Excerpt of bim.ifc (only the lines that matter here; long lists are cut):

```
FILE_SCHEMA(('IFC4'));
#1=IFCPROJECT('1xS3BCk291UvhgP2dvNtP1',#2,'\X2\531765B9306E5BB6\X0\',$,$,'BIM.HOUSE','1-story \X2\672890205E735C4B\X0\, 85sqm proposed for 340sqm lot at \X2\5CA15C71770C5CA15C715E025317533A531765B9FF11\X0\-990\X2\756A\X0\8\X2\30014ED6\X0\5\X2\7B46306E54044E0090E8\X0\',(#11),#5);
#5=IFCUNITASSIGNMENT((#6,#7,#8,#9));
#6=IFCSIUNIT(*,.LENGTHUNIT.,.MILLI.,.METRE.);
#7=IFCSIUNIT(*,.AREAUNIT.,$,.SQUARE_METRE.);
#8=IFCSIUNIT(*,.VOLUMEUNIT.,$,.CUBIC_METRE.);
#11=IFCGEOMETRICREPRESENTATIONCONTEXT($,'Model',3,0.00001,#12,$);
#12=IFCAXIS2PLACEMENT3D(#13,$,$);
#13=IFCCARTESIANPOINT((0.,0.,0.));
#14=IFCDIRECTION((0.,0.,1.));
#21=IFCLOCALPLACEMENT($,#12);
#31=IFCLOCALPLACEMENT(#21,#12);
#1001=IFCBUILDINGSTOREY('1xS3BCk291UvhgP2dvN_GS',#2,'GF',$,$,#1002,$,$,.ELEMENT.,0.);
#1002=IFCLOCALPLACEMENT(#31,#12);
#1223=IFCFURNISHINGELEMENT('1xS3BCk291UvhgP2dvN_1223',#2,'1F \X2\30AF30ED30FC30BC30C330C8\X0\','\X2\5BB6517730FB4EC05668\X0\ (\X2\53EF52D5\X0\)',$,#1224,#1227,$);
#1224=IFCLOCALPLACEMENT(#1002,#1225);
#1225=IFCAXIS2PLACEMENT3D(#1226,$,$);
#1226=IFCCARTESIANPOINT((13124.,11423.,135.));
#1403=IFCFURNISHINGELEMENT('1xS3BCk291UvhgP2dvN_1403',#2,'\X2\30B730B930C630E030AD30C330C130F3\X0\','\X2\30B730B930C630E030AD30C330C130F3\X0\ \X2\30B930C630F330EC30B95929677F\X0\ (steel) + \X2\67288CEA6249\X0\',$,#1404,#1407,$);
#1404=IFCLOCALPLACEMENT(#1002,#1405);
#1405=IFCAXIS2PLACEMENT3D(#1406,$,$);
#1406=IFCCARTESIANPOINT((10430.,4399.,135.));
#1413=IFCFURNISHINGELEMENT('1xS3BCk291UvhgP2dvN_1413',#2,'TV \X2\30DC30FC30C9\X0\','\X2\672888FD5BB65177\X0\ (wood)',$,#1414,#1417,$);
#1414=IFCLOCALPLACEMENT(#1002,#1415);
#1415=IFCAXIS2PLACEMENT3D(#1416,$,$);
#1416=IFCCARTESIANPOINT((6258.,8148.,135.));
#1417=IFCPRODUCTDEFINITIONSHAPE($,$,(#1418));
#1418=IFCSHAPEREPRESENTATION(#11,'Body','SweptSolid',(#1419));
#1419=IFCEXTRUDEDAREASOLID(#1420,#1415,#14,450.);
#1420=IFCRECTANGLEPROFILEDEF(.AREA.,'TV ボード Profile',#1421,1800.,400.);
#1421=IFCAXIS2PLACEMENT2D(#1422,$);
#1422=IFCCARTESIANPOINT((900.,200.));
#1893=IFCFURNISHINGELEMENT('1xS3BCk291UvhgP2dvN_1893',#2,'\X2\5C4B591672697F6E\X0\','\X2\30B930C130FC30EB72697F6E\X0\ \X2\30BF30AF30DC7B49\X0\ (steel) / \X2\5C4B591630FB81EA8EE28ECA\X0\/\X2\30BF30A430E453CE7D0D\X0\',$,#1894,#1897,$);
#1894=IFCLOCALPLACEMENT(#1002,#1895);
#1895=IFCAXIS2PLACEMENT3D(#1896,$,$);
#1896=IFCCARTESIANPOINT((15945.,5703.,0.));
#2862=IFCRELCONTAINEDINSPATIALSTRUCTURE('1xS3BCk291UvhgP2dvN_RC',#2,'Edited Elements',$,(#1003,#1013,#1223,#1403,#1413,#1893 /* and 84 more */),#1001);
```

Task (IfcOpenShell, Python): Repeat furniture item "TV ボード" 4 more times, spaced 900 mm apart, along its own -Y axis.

```python
import ifcopenshell
import ifcopenshell.api.geometry
import ifcopenshell.api.root
import ifcopenshell.util.element
import ifcopenshell.util.placement
import ifcopenshell.util.unit

model = ifcopenshell.open("bim.ifc")
unit_scale = ifcopenshell.util.unit.calculate_unit_scale(model)


def reuse_history(source, copy):
    """copy_class also copies each property set's owner history, people and application; keep the originals."""
    for rel in copy.IsDefinedBy:
        if rel.is_a("IfcRelDefinesByProperties") and (history := rel.RelatingPropertyDefinition.OwnerHistory):
            rel.RelatingPropertyDefinition.OwnerHistory = source.OwnerHistory
            ifcopenshell.util.element.remove_deep2(model, history)


source = model.by_guid("1xS3BCk291UvhgP2dvN_1413")
base = ifcopenshell.util.placement.get_local_placement(source.ObjectPlacement)
step = -base[:3, 1] * 0.9 / unit_scale

for i in range(1, 5):
    copy = ifcopenshell.api.root.copy_class(model, product=source)
    copy.Representation = ifcopenshell.util.element.copy_deep(
        model, source.Representation, exclude=["IfcGeometricRepresentationContext", "IfcRepresentationMap"]
    )
    reuse_history(source, copy)
    matrix = base.copy()
    matrix[:3, 3] += i * step
    print("added at", matrix[:3, 3].round(3) + 0.0)
    ifcopenshell.api.geometry.edit_object_placement(model, product=copy, matrix=matrix, is_si=False)

model.write("bim_rev.ifc")
```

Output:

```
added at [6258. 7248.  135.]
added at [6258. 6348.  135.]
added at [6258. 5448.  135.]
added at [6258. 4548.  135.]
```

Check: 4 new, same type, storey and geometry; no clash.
